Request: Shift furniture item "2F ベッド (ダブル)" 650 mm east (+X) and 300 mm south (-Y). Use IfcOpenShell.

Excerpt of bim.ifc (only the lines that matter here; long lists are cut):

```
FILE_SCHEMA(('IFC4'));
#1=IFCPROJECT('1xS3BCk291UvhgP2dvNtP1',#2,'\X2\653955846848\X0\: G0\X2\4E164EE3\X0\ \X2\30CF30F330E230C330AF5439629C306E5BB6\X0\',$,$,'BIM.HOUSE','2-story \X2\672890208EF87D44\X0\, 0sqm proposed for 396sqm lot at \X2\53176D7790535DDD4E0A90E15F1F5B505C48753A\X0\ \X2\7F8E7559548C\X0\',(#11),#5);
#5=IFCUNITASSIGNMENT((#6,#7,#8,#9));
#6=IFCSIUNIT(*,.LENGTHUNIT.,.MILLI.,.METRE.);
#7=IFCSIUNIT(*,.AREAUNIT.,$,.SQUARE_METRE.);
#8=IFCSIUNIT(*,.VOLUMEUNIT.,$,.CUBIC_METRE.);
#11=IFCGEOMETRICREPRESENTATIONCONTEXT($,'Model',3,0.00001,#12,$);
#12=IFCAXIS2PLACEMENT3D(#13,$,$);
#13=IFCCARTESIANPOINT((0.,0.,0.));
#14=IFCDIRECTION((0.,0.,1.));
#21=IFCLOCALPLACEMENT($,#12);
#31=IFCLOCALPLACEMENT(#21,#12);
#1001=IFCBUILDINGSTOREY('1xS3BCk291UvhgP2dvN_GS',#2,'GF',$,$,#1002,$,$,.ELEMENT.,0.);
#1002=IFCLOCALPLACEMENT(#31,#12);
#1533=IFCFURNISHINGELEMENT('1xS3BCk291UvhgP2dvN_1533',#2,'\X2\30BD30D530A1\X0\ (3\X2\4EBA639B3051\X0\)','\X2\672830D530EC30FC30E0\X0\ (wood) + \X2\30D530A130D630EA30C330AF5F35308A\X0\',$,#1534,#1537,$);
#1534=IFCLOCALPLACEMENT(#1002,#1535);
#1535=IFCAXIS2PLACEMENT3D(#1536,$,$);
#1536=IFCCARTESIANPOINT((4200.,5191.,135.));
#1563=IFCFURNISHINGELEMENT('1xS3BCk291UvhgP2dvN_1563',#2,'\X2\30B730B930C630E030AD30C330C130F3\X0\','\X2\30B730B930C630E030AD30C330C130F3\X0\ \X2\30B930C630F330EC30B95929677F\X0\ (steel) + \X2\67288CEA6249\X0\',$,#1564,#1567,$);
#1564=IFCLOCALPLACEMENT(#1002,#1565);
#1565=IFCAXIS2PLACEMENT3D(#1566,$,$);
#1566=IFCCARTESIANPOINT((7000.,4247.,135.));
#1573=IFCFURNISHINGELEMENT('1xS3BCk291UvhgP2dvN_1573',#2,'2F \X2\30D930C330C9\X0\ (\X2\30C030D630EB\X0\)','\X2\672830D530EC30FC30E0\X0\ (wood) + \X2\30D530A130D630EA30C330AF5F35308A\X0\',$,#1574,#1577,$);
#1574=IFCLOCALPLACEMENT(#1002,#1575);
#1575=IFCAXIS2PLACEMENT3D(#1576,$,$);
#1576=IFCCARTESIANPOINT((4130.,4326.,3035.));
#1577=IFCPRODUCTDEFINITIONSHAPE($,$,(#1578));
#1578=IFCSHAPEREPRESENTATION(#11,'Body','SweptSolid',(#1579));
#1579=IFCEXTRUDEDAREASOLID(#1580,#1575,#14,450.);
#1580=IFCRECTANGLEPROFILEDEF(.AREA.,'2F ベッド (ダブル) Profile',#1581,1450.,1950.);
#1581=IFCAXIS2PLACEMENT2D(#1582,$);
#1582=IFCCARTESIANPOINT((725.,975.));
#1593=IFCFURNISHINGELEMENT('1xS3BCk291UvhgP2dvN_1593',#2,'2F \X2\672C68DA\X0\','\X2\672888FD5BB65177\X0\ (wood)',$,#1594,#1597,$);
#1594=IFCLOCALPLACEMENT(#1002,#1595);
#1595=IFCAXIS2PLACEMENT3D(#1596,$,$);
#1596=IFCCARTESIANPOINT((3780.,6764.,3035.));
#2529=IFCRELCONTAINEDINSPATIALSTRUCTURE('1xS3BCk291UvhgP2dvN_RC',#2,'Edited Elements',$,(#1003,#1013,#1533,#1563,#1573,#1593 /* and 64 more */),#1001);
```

```python
import ifcopenshell
import ifcopenshell.api.geometry
import ifcopenshell.util.placement
import ifcopenshell.util.unit

model = ifcopenshell.open("bim.ifc")
unit_scale = ifcopenshell.util.unit.calculate_unit_scale(model)

item = model.by_guid("1xS3BCk291UvhgP2dvN_1573")
matrix = ifcopenshell.util.placement.get_local_placement(item.ObjectPlacement)
matrix[0, 3] += 0.65 / unit_scale
matrix[1, 3] -= 0.3 / unit_scale
ifcopenshell.api.geometry.edit_object_placement(model, product=item, matrix=matrix, is_si=False)

print(ifcopenshell.util.placement.get_local_placement(item.ObjectPlacement).round(3) + 0.0)

model.write("bim_v2.ifc")
```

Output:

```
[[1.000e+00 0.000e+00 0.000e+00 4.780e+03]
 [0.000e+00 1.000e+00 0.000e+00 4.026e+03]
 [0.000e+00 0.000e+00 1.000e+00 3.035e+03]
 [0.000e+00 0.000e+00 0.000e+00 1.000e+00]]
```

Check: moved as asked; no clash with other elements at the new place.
